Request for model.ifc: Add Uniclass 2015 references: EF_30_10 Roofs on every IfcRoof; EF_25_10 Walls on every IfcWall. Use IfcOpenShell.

First a look at what the model holds.

```python
import ifcopenshell

model = ifcopenshell.open("model.ifc")
print(model.schema)
print("classifications:", [c.Name for c in model.by_type("IfcClassification")])
for ifc_class in ("IfcDoor", "IfcRoof", "IfcStair", "IfcWall", "IfcWindow"):
    print(ifc_class, len(model.by_type(ifc_class)))
```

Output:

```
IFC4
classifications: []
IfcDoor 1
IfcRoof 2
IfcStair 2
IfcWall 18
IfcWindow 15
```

```python
import ifcopenshell
import ifcopenshell.api.classification

model = ifcopenshell.open("model.ifc")

system = ifcopenshell.api.classification.add_classification(model, classification="Uniclass 2015")

codes = {
    "IfcRoof": ("EF_30_10", "Roofs"),
    "IfcWall": ("EF_25_10", "Walls"),
}
for ifc_class, (code, name) in codes.items():
    products = model.by_type(ifc_class)
    ifcopenshell.api.classification.add_reference(
        model, products=products, classification=system, identification=code, name=name
    )
    print(code, len(products))

model.write("model_v2.ifc")
```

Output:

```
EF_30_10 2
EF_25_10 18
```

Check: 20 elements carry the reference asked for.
